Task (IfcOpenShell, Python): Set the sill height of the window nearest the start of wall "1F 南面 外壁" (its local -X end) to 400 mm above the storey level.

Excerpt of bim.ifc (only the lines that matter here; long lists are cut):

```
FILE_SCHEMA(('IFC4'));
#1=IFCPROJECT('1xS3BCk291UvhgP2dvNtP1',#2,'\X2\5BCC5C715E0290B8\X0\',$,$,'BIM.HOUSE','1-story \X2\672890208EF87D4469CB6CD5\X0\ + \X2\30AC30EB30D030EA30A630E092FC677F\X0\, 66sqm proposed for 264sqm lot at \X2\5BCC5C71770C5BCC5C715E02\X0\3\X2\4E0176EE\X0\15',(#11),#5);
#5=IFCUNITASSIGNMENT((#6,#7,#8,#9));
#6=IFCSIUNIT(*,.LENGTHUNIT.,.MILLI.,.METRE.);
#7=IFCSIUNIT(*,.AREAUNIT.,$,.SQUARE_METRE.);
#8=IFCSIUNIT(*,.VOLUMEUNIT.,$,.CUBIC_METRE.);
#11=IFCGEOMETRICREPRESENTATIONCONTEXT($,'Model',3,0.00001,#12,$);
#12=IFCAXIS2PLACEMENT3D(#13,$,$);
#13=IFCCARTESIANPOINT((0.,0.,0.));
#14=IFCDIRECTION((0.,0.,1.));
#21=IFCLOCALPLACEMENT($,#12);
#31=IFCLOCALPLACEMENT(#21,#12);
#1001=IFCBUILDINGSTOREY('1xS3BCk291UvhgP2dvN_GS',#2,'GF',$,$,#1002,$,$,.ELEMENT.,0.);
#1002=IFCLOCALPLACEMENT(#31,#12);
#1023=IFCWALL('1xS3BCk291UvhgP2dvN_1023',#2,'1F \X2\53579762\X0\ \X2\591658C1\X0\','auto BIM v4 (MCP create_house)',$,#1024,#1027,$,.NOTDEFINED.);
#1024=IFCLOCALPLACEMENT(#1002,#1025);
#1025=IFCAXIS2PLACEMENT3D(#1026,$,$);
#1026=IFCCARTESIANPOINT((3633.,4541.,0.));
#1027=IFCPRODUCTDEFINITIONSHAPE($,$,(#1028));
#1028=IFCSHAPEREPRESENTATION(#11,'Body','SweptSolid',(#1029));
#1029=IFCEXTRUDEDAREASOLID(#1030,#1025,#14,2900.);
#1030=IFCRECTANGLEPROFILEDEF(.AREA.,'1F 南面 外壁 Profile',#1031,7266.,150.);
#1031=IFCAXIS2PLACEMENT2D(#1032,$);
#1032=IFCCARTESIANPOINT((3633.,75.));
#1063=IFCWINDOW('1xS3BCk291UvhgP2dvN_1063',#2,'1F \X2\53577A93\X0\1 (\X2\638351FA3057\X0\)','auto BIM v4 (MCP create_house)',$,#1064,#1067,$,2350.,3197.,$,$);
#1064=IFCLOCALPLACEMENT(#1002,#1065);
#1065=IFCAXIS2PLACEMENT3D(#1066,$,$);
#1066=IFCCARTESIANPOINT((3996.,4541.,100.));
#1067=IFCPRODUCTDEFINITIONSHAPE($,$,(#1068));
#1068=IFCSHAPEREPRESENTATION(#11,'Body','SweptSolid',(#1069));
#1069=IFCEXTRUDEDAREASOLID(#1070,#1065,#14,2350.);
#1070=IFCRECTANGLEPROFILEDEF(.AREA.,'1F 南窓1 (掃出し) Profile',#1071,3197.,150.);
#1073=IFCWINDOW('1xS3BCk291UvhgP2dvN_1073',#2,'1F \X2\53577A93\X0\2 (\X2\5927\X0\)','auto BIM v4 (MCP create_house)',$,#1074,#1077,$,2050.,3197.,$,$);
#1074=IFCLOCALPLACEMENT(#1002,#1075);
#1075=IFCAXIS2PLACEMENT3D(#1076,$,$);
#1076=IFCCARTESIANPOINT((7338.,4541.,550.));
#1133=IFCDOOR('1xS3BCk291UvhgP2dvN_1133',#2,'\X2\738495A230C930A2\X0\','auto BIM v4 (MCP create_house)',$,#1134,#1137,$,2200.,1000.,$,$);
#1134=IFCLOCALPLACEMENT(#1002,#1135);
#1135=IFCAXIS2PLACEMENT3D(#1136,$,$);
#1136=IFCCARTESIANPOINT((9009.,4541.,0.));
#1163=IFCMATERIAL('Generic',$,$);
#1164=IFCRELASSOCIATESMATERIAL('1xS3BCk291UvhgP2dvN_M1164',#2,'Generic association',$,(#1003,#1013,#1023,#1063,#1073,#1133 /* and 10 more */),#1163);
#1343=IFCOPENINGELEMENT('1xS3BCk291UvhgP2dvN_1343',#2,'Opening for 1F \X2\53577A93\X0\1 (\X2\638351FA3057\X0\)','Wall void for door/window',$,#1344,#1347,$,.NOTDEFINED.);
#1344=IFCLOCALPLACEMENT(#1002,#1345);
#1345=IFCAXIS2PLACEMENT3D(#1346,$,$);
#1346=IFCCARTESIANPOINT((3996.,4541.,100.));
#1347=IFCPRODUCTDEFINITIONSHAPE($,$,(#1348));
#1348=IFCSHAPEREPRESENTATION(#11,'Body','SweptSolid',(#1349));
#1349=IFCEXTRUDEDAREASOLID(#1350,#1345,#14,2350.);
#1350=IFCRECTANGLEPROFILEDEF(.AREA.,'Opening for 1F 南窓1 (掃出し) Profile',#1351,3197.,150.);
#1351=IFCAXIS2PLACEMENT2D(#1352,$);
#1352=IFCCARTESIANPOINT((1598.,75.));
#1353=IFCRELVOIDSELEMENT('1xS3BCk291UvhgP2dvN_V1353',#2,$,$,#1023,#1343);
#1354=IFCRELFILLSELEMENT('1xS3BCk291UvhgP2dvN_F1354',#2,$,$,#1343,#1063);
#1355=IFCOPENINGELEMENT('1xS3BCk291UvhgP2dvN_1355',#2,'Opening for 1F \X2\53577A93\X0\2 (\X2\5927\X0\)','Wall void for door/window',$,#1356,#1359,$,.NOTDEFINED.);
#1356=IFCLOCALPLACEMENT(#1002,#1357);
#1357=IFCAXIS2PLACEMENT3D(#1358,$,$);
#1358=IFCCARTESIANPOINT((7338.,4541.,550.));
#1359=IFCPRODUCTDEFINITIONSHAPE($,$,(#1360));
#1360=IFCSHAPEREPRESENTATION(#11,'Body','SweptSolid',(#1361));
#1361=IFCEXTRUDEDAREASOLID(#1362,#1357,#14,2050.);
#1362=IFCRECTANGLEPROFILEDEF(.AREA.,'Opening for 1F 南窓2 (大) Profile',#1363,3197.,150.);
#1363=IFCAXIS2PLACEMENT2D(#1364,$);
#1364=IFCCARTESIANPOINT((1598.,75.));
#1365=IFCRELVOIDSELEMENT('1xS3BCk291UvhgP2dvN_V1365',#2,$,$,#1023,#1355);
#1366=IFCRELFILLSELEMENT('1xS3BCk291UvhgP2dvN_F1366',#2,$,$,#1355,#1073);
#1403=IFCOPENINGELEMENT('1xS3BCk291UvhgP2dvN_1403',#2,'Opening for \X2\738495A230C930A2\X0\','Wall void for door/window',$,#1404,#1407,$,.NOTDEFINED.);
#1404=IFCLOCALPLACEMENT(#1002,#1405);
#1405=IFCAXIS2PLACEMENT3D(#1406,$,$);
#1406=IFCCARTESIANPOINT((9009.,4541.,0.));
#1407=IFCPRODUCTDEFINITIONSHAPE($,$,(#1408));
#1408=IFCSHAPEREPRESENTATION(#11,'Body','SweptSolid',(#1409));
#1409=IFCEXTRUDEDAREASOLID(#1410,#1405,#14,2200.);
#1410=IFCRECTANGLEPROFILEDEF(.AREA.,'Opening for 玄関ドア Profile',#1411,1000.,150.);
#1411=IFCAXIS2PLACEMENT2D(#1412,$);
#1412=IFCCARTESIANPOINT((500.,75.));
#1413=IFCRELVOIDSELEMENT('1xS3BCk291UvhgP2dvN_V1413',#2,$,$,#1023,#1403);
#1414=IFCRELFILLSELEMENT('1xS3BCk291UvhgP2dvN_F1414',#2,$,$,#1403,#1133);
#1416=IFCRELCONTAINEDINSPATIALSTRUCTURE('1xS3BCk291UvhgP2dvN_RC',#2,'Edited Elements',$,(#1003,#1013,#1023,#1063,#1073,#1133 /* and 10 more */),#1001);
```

```python
import numpy as np
import ifcopenshell
import ifcopenshell.api.geometry
import ifcopenshell.geom
import ifcopenshell.util.element
import ifcopenshell.util.placement
import ifcopenshell.util.shape
import ifcopenshell.util.unit

model = ifcopenshell.open("bim.ifc")
unit_scale = ifcopenshell.util.unit.calculate_unit_scale(model)

window = model.by_guid("1xS3BCk291UvhgP2dvN_1063")
opening = window.FillsVoids[0].RelatingOpeningElement
storey = ifcopenshell.util.element.get_container(window, ifc_class="IfcBuildingStorey")
level = ifcopenshell.util.placement.get_local_placement(storey.ObjectPlacement)[2, 3]

# The opening's origin need not be at the sill, so measure its lowest point.
shape = ifcopenshell.geom.create_shape(ifcopenshell.geom.settings(), opening)
bottom = ifcopenshell.util.shape.get_shape_bottom_elevation(shape, shape.geometry) / unit_scale
dz = level + 0.4 / unit_scale - bottom

shift = np.array([0.0, 0.0, dz])
# The window is not placed relative to its opening, so move both.
for product in (opening, window):
    matrix = ifcopenshell.util.placement.get_local_placement(product.ObjectPlacement)
    matrix[:3, 3] += shift
    ifcopenshell.api.geometry.edit_object_placement(model, product=product, matrix=matrix, is_si=False)

print(f"moved by {dz * unit_scale:+.3f} m")

model.write("bim_edited.ifc")
```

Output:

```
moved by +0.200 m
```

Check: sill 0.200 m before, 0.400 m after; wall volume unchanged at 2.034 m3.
